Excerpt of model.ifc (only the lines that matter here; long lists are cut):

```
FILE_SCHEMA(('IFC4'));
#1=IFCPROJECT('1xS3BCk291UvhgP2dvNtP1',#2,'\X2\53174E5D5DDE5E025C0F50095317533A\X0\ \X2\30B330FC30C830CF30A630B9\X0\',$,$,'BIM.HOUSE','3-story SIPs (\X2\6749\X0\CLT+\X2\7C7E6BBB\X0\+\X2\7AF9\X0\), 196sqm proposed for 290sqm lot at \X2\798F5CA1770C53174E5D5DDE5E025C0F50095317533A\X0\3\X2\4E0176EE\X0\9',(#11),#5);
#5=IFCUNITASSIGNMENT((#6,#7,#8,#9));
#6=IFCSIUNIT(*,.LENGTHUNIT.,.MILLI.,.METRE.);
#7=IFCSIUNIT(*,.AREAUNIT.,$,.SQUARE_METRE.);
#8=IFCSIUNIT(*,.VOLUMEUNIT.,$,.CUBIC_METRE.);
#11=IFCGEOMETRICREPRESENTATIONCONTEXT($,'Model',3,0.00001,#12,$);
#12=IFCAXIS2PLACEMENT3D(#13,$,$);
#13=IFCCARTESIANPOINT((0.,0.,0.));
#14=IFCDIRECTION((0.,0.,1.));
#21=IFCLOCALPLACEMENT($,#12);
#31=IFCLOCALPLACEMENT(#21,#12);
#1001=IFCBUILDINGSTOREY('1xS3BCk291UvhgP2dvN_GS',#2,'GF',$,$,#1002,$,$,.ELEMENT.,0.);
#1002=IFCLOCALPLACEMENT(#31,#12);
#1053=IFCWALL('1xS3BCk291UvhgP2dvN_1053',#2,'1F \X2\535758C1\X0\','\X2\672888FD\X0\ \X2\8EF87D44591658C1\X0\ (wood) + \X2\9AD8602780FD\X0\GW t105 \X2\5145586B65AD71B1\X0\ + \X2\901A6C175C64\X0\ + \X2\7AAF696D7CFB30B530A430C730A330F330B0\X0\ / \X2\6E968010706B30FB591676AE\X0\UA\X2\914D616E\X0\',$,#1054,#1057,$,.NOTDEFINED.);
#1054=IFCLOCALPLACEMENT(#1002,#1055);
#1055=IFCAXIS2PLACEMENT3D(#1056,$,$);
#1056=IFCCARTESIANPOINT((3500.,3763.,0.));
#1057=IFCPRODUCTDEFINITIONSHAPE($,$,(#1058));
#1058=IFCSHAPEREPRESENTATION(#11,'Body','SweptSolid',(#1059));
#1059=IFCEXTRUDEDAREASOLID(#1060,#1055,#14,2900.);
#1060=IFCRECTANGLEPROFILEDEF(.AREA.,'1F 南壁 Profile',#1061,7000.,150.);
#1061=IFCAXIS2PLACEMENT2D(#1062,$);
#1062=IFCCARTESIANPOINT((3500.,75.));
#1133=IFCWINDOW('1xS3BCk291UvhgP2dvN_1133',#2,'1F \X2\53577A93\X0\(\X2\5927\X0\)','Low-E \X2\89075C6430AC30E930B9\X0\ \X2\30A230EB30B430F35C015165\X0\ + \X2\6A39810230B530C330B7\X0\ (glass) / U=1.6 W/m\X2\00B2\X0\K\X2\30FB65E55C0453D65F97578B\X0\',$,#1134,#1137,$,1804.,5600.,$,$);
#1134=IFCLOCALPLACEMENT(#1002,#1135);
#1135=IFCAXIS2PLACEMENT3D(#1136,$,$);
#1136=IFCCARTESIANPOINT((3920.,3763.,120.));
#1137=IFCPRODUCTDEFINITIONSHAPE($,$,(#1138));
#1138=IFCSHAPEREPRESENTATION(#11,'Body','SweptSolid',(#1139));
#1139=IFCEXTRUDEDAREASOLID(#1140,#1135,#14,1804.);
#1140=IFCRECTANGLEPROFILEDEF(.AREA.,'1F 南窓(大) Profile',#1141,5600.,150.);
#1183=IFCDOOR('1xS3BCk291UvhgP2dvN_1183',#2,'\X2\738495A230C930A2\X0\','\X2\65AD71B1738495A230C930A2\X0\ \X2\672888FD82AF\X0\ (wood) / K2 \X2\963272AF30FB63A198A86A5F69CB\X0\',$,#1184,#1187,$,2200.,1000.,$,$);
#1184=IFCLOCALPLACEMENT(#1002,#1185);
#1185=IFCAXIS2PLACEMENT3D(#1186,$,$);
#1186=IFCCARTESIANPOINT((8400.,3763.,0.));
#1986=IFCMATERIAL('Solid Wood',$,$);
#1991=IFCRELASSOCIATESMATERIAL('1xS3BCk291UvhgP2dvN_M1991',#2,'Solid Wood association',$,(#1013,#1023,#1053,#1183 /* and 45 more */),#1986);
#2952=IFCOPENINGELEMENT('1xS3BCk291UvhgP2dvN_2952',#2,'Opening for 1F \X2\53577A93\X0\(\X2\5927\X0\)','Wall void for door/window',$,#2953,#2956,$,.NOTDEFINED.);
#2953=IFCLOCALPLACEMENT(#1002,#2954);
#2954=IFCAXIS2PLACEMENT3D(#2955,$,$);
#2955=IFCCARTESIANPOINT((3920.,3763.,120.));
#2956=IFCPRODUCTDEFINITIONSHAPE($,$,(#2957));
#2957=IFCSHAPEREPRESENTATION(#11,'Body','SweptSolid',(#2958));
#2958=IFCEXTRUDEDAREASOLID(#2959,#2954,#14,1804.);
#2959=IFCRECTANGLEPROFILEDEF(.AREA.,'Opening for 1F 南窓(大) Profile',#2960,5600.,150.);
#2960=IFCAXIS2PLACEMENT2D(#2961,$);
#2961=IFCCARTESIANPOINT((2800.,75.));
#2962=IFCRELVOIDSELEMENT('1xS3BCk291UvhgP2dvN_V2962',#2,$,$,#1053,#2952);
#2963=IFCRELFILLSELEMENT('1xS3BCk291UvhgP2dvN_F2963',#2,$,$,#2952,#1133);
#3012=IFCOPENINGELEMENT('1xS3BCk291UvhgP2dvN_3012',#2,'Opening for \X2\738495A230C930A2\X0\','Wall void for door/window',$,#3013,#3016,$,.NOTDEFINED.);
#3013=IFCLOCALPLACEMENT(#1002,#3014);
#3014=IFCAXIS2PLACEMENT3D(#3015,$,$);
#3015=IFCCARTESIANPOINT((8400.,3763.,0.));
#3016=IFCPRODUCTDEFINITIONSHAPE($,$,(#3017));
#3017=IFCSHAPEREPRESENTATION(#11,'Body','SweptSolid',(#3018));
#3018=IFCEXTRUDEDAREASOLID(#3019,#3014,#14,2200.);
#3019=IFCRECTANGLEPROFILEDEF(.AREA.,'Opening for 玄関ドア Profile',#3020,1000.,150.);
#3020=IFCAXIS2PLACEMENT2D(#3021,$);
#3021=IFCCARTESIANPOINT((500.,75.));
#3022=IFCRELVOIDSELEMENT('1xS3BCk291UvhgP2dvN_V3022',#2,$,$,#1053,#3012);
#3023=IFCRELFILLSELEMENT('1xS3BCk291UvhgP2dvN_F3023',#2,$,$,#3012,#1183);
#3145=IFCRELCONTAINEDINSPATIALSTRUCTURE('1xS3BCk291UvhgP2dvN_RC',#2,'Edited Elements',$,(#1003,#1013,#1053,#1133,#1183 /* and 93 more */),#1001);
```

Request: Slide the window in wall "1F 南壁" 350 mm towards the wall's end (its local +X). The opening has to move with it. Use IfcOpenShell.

```python
import ifcopenshell
import ifcopenshell.api.geometry
import ifcopenshell.util.placement
import ifcopenshell.util.unit

model = ifcopenshell.open("model.ifc")
unit_scale = ifcopenshell.util.unit.calculate_unit_scale(model)

window = model.by_id(1133)
opening = window.FillsVoids[0].RelatingOpeningElement
wall = opening.VoidsElements[0].RelatingBuildingElement

wall_matrix = ifcopenshell.util.placement.get_local_placement(wall.ObjectPlacement)
shift = wall_matrix[:3, 0] * 0.35 / unit_scale
before = ifcopenshell.util.placement.get_local_placement(window.ObjectPlacement)[:3, 3].copy()

# The window is not placed relative to its opening, so move both.
for product in (opening, window):
    matrix = ifcopenshell.util.placement.get_local_placement(product.ObjectPlacement)
    matrix[:3, 3] += shift
    ifcopenshell.api.geometry.edit_object_placement(model, product=product, matrix=matrix, is_si=False)

after = ifcopenshell.util.placement.get_local_placement(window.ObjectPlacement)[:3, 3]
print("window moved by", (after - before).round(3) + 0.0)

model.write("model-out.ifc")
```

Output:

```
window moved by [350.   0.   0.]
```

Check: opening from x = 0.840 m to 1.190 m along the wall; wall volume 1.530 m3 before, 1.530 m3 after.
